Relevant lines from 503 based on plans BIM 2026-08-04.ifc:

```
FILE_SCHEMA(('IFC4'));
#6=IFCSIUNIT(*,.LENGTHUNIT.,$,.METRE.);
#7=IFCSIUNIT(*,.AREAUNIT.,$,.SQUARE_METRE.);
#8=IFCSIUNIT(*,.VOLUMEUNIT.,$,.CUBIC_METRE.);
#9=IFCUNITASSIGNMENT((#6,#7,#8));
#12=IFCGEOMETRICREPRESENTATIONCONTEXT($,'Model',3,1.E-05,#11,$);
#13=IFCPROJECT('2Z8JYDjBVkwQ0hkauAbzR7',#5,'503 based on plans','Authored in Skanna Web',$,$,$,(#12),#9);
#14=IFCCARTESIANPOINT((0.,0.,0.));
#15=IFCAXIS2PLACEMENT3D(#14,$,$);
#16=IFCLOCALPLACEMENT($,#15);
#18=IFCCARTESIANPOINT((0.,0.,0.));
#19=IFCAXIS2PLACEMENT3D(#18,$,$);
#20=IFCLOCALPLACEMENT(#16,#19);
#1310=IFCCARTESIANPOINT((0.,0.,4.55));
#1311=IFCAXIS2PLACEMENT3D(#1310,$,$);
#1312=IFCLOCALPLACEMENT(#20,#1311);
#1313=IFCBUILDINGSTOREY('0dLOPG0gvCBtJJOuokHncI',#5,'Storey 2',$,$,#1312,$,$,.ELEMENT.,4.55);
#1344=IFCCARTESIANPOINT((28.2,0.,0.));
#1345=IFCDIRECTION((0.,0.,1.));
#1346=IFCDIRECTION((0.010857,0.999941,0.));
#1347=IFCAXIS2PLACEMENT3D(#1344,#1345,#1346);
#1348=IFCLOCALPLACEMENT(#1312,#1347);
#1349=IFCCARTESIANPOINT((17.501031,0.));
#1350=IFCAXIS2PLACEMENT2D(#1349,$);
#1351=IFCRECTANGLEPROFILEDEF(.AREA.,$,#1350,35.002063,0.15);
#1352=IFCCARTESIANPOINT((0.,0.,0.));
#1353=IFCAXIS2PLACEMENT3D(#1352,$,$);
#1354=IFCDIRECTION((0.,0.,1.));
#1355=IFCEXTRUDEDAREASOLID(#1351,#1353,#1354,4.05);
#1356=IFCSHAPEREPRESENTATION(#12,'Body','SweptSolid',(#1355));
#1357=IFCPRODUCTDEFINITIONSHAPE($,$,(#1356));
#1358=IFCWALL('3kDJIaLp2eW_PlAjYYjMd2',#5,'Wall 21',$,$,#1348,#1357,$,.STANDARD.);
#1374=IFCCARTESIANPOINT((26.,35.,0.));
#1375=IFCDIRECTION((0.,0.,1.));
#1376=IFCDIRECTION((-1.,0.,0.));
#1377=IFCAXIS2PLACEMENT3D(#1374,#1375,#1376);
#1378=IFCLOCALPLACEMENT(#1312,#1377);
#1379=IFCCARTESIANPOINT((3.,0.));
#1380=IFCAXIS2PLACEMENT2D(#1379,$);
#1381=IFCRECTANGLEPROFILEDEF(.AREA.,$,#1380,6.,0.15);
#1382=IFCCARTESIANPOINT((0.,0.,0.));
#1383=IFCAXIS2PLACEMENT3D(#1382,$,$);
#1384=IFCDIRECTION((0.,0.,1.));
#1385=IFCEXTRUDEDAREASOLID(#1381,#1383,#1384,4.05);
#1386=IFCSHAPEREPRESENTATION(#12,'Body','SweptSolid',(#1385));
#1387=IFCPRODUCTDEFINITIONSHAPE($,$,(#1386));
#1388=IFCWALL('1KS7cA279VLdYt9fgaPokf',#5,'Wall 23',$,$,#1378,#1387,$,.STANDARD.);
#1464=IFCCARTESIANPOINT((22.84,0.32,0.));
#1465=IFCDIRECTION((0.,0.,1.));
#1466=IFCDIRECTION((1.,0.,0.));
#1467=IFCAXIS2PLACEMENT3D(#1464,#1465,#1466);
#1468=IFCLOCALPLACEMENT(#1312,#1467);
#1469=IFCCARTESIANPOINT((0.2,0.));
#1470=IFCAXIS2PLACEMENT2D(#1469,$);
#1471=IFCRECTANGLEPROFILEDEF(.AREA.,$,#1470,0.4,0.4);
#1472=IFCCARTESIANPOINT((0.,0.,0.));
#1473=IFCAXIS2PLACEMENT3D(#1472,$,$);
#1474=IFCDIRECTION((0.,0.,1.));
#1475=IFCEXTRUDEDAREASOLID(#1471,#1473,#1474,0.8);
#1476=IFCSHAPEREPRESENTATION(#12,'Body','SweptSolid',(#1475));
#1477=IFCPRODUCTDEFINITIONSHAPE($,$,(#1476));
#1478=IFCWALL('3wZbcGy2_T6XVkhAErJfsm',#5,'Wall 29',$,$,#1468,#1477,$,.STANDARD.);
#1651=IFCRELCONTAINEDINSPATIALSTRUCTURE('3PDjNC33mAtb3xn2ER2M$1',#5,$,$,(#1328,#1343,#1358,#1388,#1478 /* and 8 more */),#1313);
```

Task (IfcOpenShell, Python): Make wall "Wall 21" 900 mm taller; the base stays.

```python
import ifcopenshell
import ifcopenshell.geom
import ifcopenshell.util.shape
import ifcopenshell.util.unit

model = ifcopenshell.open("503 based on plans BIM 2026-08-04.ifc")
unit_scale = ifcopenshell.util.unit.calculate_unit_scale(model)
settings = ifcopenshell.geom.settings()


def volume(element):
    """Net volume in cubic metres, openings subtracted."""
    shape = ifcopenshell.geom.create_shape(settings, element)
    return ifcopenshell.util.shape.get_volume(shape.geometry)


wall = model.by_guid("3kDJIaLp2eW_PlAjYYjMd2")
before = volume(wall)

body = next(r for r in wall.Representation.Representations if r.RepresentationIdentifier == "Body")
solid = body.Items[0]
old_height = solid.Depth
solid.Depth += 0.9 / unit_scale
after = volume(wall)

print(f"height {old_height:g} -> {solid.Depth:g}, volume {before:.3f} -> {after:.3f} m3")

model.write("503 based on plans BIM 2026-08-04-out.ifc")
```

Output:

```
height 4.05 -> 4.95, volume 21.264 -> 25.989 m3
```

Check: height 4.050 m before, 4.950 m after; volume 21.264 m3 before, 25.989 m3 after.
